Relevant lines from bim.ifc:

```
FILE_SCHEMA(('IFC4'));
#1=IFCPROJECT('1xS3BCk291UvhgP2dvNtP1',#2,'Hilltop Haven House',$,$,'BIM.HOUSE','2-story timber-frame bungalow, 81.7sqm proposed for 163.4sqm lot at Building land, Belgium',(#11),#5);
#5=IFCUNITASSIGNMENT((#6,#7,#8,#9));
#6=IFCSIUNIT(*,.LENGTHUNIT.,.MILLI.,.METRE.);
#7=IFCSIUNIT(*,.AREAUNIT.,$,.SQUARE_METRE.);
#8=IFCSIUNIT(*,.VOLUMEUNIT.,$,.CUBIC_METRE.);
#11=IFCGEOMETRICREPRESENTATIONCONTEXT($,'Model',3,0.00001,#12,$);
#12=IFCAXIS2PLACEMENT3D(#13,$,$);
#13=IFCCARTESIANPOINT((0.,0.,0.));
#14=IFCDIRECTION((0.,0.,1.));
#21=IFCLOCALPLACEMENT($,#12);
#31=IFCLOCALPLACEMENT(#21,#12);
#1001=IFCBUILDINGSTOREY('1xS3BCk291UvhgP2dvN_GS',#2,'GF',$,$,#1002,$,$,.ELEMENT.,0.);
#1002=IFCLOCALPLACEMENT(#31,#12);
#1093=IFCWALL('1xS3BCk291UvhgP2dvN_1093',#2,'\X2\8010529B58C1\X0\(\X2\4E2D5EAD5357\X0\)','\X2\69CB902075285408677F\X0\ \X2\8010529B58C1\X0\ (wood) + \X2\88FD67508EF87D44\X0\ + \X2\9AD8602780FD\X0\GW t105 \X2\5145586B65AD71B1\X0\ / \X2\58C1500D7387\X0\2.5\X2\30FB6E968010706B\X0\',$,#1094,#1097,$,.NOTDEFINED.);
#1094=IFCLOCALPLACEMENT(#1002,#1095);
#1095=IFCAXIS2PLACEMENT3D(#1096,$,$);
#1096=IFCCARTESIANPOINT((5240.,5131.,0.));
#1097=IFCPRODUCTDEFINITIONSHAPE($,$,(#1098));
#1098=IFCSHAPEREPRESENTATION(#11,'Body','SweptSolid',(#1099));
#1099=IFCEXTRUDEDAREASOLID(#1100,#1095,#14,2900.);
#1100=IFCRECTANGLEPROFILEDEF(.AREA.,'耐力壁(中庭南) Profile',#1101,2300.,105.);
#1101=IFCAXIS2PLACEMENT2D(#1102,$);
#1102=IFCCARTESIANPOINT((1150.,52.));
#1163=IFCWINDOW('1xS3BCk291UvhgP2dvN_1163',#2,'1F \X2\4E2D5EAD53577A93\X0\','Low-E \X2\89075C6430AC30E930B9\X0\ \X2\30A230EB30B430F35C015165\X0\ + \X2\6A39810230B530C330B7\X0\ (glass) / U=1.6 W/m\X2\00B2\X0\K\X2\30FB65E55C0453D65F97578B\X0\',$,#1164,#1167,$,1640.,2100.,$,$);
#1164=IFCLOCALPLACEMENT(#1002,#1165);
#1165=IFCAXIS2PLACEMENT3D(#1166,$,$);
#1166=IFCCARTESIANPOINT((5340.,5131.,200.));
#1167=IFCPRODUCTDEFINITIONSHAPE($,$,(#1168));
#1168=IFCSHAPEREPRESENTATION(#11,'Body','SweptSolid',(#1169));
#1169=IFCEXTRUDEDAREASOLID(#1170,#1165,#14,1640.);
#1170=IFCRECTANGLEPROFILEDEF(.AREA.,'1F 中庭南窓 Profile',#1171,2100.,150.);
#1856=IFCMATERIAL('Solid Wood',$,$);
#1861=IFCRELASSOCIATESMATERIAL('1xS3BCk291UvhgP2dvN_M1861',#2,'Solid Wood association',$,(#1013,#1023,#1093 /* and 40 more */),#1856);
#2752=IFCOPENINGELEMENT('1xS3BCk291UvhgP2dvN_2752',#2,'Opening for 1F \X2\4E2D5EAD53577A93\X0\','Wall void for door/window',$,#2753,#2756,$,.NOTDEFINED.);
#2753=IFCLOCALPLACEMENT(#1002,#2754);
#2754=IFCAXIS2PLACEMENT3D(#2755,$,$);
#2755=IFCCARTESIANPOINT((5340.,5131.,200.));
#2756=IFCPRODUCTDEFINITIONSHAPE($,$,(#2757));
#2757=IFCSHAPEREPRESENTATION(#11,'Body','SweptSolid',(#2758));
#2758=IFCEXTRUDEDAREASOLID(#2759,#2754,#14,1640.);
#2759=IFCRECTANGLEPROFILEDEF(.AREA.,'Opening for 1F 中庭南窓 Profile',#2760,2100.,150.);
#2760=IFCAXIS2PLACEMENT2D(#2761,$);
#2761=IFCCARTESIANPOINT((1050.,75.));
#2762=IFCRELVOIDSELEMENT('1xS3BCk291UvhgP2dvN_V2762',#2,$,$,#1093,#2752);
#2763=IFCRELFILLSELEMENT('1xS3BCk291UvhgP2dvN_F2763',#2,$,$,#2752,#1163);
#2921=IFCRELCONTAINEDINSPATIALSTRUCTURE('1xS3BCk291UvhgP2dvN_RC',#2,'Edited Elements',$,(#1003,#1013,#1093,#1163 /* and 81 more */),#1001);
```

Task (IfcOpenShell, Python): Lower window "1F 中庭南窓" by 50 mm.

```python
import numpy as np
import ifcopenshell
import ifcopenshell.api.geometry
import ifcopenshell.util.placement
import ifcopenshell.util.unit

model = ifcopenshell.open("bim.ifc")
unit_scale = ifcopenshell.util.unit.calculate_unit_scale(model)

window = model.by_guid("1xS3BCk291UvhgP2dvN_1163")
opening = window.FillsVoids[0].RelatingOpeningElement
dz = -50.0

shift = np.array([0.0, 0.0, dz])
# The window is not placed relative to its opening, so move both.
for product in (opening, window):
    matrix = ifcopenshell.util.placement.get_local_placement(product.ObjectPlacement)
    matrix[:3, 3] += shift
    ifcopenshell.api.geometry.edit_object_placement(model, product=product, matrix=matrix, is_si=False)

print(f"moved by {dz * unit_scale:+.3f} m")

model.write("bim_rev.ifc")
```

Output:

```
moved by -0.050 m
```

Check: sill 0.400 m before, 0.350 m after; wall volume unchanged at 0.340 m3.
